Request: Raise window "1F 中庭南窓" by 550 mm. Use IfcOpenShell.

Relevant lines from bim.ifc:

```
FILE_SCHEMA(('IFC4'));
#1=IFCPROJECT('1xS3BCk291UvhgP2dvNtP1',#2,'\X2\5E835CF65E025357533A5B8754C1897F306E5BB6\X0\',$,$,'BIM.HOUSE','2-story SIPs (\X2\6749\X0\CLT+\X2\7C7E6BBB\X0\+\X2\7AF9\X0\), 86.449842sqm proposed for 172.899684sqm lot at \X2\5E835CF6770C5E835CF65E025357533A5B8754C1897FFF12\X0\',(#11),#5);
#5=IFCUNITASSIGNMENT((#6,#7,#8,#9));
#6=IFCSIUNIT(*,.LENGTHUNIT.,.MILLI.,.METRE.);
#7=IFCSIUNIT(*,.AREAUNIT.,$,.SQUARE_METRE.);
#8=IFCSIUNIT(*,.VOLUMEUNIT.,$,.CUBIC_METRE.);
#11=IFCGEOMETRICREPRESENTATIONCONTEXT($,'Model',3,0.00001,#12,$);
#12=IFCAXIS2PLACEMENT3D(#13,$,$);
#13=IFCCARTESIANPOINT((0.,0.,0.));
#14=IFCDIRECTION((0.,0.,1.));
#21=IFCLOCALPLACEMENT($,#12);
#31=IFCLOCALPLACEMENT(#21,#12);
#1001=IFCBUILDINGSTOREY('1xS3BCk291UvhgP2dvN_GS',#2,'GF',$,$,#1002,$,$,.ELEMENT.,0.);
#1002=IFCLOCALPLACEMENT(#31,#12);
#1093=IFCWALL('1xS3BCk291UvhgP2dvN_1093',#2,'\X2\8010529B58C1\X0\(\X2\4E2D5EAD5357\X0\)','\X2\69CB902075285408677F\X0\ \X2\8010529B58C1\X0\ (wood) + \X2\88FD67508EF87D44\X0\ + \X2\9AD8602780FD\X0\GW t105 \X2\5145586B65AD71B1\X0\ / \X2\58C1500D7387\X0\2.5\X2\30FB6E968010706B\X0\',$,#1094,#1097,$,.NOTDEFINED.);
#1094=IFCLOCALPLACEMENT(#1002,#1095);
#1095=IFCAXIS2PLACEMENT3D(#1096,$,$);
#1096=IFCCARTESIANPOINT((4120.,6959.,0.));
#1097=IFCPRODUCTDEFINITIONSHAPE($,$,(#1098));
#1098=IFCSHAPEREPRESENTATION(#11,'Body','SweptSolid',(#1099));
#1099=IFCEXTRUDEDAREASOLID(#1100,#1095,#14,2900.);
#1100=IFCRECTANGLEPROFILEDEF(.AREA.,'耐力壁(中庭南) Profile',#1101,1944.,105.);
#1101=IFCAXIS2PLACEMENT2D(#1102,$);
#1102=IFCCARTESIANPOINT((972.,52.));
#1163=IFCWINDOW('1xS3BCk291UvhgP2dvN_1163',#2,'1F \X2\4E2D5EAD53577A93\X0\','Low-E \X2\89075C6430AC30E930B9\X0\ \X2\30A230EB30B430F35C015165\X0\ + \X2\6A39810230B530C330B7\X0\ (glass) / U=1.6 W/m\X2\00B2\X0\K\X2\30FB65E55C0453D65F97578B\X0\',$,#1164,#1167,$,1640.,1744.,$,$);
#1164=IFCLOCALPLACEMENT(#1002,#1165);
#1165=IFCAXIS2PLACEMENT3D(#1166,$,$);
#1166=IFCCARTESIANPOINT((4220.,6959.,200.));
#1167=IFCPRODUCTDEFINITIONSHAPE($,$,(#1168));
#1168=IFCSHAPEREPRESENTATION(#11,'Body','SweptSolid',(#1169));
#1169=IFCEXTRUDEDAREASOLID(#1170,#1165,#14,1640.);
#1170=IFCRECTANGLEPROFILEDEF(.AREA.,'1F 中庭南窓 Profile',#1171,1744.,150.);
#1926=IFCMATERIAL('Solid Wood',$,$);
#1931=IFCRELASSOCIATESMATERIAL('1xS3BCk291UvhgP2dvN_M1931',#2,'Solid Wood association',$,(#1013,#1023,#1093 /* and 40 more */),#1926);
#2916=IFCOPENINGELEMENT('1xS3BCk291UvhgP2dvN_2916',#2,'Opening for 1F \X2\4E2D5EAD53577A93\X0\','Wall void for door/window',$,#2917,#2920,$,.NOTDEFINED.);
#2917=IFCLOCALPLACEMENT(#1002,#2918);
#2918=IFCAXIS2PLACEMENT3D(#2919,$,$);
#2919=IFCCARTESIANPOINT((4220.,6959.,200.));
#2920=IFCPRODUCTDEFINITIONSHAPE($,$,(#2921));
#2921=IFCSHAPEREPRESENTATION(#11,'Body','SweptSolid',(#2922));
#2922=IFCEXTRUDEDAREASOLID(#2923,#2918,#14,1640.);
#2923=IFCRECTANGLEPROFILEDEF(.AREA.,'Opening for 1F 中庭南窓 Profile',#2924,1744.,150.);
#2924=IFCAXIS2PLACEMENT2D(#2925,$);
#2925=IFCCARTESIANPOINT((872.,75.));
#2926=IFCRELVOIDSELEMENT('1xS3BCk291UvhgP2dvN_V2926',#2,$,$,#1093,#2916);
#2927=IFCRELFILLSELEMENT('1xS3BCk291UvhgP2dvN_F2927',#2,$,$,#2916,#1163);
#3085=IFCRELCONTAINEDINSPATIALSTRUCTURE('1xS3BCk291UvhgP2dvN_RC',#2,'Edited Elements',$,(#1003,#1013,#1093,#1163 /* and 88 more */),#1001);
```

```python
import numpy as np
import ifcopenshell
import ifcopenshell.api.geometry
import ifcopenshell.util.placement
import ifcopenshell.util.unit

model = ifcopenshell.open("bim.ifc")
unit_scale = ifcopenshell.util.unit.calculate_unit_scale(model)

window = model.by_guid("1xS3BCk291UvhgP2dvN_1163")
opening = window.FillsVoids[0].RelatingOpeningElement
dz = 550.0

shift = np.array([0.0, 0.0, dz])
# The window is not placed relative to its opening, so move both.
for product in (opening, window):
    matrix = ifcopenshell.util.placement.get_local_placement(product.ObjectPlacement)
    matrix[:3, 3] += shift
    ifcopenshell.api.geometry.edit_object_placement(model, product=product, matrix=matrix, is_si=False)

print(f"moved by {dz * unit_scale:+.3f} m")

model.write("bim_updated.ifc")
```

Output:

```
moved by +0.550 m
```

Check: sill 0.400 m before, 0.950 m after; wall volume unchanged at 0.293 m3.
